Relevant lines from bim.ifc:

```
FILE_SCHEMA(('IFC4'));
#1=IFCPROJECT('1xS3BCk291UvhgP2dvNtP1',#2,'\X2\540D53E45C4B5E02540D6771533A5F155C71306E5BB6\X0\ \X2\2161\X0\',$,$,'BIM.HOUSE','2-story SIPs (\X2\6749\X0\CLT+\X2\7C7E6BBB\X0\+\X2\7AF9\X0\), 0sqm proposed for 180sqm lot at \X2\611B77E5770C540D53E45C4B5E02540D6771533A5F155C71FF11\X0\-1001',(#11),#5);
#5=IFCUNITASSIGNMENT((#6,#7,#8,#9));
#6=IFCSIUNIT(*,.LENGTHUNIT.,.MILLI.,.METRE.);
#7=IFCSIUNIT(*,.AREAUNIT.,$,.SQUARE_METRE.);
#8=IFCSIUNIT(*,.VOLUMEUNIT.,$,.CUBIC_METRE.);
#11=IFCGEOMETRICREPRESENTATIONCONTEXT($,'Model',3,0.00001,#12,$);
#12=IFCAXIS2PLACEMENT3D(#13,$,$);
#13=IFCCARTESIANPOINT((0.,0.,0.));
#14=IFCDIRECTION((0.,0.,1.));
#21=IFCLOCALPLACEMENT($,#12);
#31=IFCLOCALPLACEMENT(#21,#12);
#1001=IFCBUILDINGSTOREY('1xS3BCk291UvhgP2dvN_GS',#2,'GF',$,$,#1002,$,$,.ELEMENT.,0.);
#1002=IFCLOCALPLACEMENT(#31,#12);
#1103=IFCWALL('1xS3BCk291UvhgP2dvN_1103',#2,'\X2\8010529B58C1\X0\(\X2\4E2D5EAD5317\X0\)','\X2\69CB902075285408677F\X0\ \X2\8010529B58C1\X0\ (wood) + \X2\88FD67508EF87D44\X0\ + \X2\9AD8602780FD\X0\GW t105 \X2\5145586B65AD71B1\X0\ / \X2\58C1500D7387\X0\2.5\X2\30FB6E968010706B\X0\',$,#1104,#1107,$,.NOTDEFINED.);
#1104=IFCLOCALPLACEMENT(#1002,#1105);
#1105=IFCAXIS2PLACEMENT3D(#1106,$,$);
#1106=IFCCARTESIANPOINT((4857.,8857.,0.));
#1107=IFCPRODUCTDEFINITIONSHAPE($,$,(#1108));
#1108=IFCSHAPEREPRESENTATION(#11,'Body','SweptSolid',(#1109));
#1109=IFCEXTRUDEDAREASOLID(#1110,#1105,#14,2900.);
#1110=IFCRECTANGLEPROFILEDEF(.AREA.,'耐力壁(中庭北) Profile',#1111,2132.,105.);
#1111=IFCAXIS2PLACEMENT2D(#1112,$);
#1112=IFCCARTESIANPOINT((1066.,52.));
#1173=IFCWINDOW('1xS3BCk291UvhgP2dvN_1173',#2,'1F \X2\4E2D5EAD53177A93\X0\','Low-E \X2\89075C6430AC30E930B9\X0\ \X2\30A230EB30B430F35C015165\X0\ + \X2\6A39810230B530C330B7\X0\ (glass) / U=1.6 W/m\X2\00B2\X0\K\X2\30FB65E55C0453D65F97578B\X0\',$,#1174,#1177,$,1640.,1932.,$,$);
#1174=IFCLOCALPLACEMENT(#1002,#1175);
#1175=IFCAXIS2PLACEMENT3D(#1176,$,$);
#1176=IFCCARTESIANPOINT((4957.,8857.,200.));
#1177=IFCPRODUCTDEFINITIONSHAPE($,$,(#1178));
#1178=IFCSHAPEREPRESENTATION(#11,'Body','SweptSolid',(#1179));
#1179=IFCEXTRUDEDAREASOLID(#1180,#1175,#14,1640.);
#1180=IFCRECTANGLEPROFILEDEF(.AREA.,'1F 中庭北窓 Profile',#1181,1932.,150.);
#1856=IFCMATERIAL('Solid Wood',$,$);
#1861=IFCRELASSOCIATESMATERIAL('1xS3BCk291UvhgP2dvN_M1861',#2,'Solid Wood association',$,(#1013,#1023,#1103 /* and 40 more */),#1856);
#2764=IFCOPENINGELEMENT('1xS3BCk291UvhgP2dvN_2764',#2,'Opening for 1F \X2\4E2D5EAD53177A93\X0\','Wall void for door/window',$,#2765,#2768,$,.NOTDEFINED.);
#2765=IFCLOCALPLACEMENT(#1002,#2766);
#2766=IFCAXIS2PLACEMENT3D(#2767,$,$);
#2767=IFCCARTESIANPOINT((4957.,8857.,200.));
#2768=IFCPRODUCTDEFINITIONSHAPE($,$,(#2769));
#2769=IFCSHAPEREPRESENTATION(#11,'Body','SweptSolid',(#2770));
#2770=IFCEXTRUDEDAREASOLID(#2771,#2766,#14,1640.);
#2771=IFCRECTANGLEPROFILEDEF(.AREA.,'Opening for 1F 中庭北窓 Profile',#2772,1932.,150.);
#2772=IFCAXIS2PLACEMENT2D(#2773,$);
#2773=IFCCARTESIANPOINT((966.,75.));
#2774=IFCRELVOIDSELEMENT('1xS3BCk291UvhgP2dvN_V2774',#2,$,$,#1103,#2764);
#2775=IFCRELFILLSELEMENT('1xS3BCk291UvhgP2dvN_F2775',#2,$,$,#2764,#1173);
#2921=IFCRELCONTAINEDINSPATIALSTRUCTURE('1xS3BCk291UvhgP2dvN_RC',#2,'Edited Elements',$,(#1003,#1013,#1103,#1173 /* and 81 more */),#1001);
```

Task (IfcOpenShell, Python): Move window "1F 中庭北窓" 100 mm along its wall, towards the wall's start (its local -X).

```python
import ifcopenshell
import ifcopenshell.api.geometry
import ifcopenshell.util.placement

model = ifcopenshell.open("bim.ifc")

window = model.by_guid("1xS3BCk291UvhgP2dvN_1173")
opening = window.FillsVoids[0].RelatingOpeningElement
wall = opening.VoidsElements[0].RelatingBuildingElement

wall_matrix = ifcopenshell.util.placement.get_local_placement(wall.ObjectPlacement)
shift = wall_matrix[:3, 0] * -100.0
before = ifcopenshell.util.placement.get_local_placement(window.ObjectPlacement)[:3, 3].copy()

# The window is not placed relative to its opening, so move both.
for product in (opening, window):
    matrix = ifcopenshell.util.placement.get_local_placement(product.ObjectPlacement)
    matrix[:3, 3] += shift
    ifcopenshell.api.geometry.edit_object_placement(model, product=product, matrix=matrix, is_si=False)

after = ifcopenshell.util.placement.get_local_placement(window.ObjectPlacement)[:3, 3]
print("window moved by", (after - before).round(3) + 0.0)

model.write("bim_edited.ifc")
```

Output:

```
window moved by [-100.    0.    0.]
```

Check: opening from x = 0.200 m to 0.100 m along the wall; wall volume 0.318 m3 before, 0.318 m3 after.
